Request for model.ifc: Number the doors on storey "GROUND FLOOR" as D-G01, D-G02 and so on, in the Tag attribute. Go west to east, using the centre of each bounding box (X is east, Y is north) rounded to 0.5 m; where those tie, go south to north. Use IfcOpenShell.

First a look at what the model holds.

```python
import ifcopenshell
import ifcopenshell.util.element
import ifcopenshell.util.placement

model = ifcopenshell.open("model.ifc")
print(model.schema)
storey = next(s for s in model.by_type("IfcBuildingStorey") if s.Name == "GROUND FLOOR")
doors = [e for e in ifcopenshell.util.element.get_decomposition(storey) if e.is_a("IfcDoor")]
for e in sorted(doors, key=lambda e: e.id()):
    origin = ifcopenshell.util.placement.get_local_placement(e.ObjectPlacement)[:3, 3]
    print(e.id(), e.Tag, e.Name, origin.round(2) + 0.0, sep=" | ")
```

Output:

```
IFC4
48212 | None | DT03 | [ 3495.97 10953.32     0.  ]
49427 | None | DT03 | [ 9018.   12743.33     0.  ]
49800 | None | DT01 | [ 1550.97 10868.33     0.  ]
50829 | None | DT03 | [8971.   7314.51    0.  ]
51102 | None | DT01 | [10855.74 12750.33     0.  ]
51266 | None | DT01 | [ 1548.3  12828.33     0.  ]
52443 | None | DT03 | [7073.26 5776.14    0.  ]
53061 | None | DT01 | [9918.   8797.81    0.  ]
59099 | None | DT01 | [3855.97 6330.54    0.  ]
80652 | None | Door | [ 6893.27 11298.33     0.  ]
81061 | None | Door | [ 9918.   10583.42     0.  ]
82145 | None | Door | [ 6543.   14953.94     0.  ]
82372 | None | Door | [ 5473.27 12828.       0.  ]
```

```python
import ifcopenshell
import ifcopenshell.geom
import ifcopenshell.util.element
import ifcopenshell.util.shape

model = ifcopenshell.open("model.ifc")
settings = ifcopenshell.geom.settings()
settings.set("use-world-coords", True)


def centre(element):
    shape = ifcopenshell.geom.create_shape(settings, element)
    return ifcopenshell.util.shape.get_bbox_centroid(shape.geometry)


storey = next(s for s in model.by_type("IfcBuildingStorey") if s.Name == "GROUND FLOOR")
doors = [e for e in ifcopenshell.util.element.get_decomposition(storey) if e.is_a("IfcDoor")]

# Insertion points can sit at a corner or the storey origin, so sort by the geometry (in metres).
centres = {e: centre(e) for e in doors}
doors.sort(key=lambda e: (round(centres[e][0] / 0.5), centres[e][1]))

for i, e in enumerate(doors, start=1):
    number = f"D-G{i:02d}"
    e.Tag = number
    print(e.id(), number)

model.write("model_v2.ifc")
```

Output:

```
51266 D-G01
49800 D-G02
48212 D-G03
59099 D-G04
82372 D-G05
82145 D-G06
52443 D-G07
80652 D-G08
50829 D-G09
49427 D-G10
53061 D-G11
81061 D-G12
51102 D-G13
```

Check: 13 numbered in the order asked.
